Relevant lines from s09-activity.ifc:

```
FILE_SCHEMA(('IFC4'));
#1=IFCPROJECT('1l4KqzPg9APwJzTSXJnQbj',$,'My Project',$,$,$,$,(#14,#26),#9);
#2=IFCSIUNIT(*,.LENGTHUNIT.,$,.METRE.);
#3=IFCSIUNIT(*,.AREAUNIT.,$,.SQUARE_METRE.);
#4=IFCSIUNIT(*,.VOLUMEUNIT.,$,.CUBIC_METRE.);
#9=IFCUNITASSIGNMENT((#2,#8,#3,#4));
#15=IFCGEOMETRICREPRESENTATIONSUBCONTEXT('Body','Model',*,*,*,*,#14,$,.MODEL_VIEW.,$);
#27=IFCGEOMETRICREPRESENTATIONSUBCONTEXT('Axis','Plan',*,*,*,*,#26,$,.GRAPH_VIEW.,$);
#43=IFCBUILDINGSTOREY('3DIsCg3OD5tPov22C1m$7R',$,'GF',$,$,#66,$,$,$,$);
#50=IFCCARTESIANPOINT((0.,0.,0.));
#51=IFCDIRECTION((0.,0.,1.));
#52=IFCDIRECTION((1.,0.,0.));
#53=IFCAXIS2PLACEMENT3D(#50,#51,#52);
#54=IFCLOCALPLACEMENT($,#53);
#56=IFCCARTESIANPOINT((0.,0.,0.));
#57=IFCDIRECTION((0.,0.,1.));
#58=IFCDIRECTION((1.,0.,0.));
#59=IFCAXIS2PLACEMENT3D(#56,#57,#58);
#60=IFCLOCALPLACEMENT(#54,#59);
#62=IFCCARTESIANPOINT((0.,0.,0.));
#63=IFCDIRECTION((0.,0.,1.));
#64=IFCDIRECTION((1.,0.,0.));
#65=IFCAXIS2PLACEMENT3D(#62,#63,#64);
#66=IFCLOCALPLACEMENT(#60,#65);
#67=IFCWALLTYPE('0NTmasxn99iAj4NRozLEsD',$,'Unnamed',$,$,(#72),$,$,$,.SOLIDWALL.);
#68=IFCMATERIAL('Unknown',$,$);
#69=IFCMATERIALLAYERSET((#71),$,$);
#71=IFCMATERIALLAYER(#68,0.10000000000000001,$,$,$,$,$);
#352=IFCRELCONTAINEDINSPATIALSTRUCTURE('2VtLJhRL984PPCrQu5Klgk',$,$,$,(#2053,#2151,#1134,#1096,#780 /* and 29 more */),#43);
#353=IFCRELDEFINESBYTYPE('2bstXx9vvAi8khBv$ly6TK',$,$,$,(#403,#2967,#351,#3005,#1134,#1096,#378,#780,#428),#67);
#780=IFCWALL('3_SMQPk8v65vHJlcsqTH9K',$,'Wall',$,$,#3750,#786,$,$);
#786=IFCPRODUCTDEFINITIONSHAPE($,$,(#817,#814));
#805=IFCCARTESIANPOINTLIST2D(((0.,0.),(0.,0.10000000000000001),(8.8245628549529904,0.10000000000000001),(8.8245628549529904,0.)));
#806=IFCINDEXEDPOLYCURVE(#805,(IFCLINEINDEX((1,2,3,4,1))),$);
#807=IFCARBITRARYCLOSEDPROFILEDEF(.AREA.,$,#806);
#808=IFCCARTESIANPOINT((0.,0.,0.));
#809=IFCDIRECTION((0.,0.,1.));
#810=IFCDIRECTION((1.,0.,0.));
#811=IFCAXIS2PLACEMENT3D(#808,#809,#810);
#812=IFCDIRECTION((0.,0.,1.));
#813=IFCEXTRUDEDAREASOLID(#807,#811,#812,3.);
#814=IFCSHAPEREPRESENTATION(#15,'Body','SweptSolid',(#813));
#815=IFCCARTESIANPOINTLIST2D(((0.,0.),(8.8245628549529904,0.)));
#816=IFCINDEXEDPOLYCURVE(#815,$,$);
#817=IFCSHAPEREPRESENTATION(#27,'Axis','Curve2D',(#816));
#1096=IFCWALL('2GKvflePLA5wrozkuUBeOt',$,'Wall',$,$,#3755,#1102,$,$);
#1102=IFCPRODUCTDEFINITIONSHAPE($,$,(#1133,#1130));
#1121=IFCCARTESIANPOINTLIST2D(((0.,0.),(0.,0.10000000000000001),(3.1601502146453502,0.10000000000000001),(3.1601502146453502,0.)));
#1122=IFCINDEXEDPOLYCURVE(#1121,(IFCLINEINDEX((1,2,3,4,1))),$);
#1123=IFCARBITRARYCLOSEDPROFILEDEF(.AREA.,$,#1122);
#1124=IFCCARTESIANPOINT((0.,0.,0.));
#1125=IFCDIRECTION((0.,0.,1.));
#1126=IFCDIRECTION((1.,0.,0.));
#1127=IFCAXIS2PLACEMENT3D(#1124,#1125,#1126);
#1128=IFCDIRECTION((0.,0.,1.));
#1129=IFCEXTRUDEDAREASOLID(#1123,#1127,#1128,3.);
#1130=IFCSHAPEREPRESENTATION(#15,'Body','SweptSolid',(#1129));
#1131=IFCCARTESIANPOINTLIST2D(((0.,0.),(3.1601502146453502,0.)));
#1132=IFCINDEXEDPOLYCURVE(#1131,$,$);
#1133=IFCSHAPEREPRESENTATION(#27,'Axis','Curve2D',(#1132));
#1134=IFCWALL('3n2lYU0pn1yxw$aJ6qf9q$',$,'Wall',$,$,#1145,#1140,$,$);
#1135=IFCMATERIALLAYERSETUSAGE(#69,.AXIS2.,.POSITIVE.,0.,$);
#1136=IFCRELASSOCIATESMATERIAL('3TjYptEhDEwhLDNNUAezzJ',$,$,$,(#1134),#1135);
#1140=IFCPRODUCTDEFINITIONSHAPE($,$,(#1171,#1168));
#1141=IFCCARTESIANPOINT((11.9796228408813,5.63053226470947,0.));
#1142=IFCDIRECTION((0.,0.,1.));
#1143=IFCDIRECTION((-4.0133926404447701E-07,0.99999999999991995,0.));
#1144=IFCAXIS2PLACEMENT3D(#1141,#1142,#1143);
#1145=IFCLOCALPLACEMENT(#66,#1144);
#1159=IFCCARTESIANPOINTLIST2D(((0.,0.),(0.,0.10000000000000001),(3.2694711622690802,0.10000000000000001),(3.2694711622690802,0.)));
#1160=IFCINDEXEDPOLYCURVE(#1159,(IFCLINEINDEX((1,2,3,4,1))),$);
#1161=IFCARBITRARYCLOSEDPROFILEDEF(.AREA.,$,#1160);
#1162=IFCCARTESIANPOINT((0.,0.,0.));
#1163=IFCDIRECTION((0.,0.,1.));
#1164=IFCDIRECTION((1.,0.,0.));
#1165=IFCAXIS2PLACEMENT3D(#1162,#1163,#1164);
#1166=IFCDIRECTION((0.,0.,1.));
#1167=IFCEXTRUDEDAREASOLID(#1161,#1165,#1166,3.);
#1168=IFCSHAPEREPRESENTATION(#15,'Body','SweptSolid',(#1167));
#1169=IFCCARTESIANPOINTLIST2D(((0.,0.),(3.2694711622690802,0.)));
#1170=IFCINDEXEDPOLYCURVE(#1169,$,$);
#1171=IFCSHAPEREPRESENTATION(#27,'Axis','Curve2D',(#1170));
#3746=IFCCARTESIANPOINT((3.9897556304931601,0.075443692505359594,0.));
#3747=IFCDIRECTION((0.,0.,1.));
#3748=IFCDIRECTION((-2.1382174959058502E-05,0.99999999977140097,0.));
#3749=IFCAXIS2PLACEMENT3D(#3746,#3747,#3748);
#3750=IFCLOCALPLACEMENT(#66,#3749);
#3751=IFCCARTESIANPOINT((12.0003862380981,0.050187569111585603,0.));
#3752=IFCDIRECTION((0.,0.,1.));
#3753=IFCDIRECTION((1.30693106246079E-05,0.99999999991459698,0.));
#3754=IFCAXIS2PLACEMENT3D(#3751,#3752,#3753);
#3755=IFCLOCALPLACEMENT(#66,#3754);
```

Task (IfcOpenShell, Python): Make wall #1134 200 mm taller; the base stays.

```python
import ifcopenshell
import ifcopenshell.geom
import ifcopenshell.util.representation
import ifcopenshell.util.shape
import ifcopenshell.util.unit

model = ifcopenshell.open("s09-activity.ifc")
unit_scale = ifcopenshell.util.unit.calculate_unit_scale(model)
settings = ifcopenshell.geom.settings()


def volume(element):
    """Net volume in cubic metres, openings subtracted."""
    shape = ifcopenshell.geom.create_shape(settings, element)
    return ifcopenshell.util.shape.get_volume(shape.geometry)


wall = model.by_id(1134)
before = volume(wall)

body = ifcopenshell.util.representation.get_representation(wall, "Model", "Body")
solid = body.Items[0]
old_height = solid.Depth
solid.Depth += 0.2 / unit_scale
after = volume(wall)

print(f"height {old_height:g} -> {solid.Depth:g}, volume {before:.3f} -> {after:.3f} m3")

model.write("s09-activity_updated.ifc")
```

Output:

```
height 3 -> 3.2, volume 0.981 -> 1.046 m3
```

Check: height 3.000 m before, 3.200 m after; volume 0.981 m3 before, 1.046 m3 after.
